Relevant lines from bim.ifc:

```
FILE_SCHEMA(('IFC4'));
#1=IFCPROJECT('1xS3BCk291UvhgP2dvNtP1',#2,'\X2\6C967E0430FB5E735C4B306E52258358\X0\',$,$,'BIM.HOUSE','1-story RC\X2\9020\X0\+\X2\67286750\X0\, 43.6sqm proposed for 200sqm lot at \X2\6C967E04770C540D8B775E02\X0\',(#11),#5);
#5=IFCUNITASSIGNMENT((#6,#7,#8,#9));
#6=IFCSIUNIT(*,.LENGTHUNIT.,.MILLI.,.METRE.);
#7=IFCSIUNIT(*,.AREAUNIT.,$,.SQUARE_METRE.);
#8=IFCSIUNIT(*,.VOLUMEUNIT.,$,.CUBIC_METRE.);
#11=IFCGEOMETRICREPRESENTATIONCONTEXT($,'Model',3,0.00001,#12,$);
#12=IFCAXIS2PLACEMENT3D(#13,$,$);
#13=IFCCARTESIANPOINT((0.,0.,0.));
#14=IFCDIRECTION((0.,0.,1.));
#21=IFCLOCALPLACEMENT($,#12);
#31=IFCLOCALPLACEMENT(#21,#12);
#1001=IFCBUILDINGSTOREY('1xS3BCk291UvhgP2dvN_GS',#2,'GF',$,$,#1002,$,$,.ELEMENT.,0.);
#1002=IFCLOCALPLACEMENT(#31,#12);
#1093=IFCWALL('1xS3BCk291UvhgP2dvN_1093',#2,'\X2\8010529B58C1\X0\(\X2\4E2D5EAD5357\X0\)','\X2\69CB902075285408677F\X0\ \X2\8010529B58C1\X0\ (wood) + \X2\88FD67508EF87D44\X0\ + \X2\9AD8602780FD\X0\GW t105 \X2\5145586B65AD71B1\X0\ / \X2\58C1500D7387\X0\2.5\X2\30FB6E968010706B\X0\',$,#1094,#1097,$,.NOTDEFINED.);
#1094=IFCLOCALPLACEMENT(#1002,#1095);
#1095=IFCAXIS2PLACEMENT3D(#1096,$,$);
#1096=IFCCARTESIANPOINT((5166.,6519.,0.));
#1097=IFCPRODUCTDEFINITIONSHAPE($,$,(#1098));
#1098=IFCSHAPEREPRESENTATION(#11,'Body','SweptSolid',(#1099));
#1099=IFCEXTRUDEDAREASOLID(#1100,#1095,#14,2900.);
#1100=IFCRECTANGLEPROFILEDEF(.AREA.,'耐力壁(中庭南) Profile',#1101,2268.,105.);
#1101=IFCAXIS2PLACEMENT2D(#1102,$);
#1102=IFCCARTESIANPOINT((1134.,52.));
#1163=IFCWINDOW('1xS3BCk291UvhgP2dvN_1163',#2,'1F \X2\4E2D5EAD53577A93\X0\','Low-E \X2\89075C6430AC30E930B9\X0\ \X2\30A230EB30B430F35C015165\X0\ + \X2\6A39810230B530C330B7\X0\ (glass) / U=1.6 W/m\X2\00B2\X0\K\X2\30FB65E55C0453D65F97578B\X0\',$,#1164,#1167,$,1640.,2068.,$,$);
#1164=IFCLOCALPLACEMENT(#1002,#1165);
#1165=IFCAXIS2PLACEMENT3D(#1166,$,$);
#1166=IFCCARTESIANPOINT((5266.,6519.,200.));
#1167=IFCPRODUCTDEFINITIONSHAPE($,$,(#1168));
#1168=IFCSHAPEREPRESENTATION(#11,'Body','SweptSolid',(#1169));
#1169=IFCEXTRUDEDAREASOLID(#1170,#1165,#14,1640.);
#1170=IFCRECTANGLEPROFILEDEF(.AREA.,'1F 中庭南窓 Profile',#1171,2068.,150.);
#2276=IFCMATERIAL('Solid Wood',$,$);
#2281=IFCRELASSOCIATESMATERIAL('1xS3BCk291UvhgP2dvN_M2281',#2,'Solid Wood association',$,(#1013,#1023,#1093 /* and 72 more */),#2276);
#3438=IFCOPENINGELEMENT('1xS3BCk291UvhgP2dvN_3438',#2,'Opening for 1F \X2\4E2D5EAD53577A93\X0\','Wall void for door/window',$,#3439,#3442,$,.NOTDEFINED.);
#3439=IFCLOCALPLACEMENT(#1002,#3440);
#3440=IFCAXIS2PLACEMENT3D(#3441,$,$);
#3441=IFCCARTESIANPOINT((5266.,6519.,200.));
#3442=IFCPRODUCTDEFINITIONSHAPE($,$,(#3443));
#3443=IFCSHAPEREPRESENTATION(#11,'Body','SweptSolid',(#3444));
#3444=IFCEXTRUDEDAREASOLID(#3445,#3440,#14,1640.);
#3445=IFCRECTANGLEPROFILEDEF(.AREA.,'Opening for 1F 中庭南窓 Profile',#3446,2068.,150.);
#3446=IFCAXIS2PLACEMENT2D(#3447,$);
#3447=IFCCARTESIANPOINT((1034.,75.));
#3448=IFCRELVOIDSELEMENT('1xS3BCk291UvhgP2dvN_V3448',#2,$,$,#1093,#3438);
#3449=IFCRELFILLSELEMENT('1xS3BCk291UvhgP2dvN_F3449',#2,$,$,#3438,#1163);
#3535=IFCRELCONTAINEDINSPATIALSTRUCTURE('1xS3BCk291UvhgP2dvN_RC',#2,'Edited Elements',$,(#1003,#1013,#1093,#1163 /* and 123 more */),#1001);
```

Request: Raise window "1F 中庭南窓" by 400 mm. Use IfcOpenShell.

```python
import numpy as np
import ifcopenshell
import ifcopenshell.api.geometry
import ifcopenshell.util.placement
import ifcopenshell.util.unit

model = ifcopenshell.open("bim.ifc")
unit_scale = ifcopenshell.util.unit.calculate_unit_scale(model)

window = model.by_id(1163)
opening = window.FillsVoids[0].RelatingOpeningElement
dz = 0.4 / unit_scale

shift = np.array([0.0, 0.0, dz])
# The window is not placed relative to its opening, so move both.
for product in (opening, window):
    matrix = ifcopenshell.util.placement.get_local_placement(product.ObjectPlacement)
    matrix[:3, 3] += shift
    ifcopenshell.api.geometry.edit_object_placement(model, product=product, matrix=matrix, is_si=False)

print(f"moved by {dz * unit_scale:+.3f} m")

model.write("bim_v2.ifc")
```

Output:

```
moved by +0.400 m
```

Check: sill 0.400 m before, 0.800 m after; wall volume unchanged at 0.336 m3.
